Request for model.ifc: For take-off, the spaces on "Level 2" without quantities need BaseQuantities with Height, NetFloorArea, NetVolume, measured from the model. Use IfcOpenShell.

First a look at what the model holds.

```python
import ifcopenshell
import ifcopenshell.util.element
import ifcopenshell.util.unit

model = ifcopenshell.open("model.ifc")
print(model.schema)
for unit_type in ("LENGTHUNIT", "AREAUNIT", "VOLUMEUNIT"):
    print(unit_type, ifcopenshell.util.unit.calculate_unit_scale(model, unit_type))
storey = next(s for s in model.by_type("IfcBuildingStorey") if s.Name == "Level 2")
spaces = [e for e in ifcopenshell.util.element.get_decomposition(storey) if e.is_a("IfcSpace")]
for e in sorted(spaces, key=lambda e: e.id()):
    print(e.id(), e.is_a(), e.Name, list(ifcopenshell.util.element.get_psets(e, qtos_only=True)), sep=" | ")
```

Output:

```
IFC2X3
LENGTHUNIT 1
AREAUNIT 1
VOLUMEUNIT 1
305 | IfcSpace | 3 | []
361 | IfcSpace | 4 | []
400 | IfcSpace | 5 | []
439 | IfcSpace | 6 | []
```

```python
import ifcopenshell
import ifcopenshell.api.pset
import ifcopenshell.geom
import ifcopenshell.util.element
import ifcopenshell.util.shape
import ifcopenshell.util.unit

model = ifcopenshell.open("model.ifc")
unit_scale = ifcopenshell.util.unit.calculate_unit_scale(model)
area_scale = ifcopenshell.util.unit.calculate_unit_scale(model, "AREAUNIT")
volume_scale = ifcopenshell.util.unit.calculate_unit_scale(model, "VOLUMEUNIT")
settings = ifcopenshell.geom.settings()

storey = next(s for s in model.by_type("IfcBuildingStorey") if s.Name == "Level 2")
spaces = [e for e in ifcopenshell.util.element.get_decomposition(storey) if e.is_a("IfcSpace")]

for e in sorted(spaces, key=lambda e: e.id()):
    if ifcopenshell.util.element.get_psets(e, qtos_only=True, should_inherit=False):
        continue
    # Geometry comes back in metres, in the element's own axes.
    shape = ifcopenshell.geom.create_shape(settings, e)
    values = {
        "Height": ifcopenshell.util.shape.get_z(shape.geometry) / unit_scale,
        "NetFloorArea": ifcopenshell.util.shape.get_footprint_area(shape.geometry) / area_scale,
        "NetVolume": ifcopenshell.util.shape.get_volume(shape.geometry) / volume_scale,
    }
    qto = ifcopenshell.api.pset.add_qto(model, product=e, name="BaseQuantities")
    ifcopenshell.api.pset.edit_qto(model, qto=qto, properties=values)
    print(e.id(), {k: round(v, 3) for k, v in values.items()})

model.write("model_v2.ifc")
```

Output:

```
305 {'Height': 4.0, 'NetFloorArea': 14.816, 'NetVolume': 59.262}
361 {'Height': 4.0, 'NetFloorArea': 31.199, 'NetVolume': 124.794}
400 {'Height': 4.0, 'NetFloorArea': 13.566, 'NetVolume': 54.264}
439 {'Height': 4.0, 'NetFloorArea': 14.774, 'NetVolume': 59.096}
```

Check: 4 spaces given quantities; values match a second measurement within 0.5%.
